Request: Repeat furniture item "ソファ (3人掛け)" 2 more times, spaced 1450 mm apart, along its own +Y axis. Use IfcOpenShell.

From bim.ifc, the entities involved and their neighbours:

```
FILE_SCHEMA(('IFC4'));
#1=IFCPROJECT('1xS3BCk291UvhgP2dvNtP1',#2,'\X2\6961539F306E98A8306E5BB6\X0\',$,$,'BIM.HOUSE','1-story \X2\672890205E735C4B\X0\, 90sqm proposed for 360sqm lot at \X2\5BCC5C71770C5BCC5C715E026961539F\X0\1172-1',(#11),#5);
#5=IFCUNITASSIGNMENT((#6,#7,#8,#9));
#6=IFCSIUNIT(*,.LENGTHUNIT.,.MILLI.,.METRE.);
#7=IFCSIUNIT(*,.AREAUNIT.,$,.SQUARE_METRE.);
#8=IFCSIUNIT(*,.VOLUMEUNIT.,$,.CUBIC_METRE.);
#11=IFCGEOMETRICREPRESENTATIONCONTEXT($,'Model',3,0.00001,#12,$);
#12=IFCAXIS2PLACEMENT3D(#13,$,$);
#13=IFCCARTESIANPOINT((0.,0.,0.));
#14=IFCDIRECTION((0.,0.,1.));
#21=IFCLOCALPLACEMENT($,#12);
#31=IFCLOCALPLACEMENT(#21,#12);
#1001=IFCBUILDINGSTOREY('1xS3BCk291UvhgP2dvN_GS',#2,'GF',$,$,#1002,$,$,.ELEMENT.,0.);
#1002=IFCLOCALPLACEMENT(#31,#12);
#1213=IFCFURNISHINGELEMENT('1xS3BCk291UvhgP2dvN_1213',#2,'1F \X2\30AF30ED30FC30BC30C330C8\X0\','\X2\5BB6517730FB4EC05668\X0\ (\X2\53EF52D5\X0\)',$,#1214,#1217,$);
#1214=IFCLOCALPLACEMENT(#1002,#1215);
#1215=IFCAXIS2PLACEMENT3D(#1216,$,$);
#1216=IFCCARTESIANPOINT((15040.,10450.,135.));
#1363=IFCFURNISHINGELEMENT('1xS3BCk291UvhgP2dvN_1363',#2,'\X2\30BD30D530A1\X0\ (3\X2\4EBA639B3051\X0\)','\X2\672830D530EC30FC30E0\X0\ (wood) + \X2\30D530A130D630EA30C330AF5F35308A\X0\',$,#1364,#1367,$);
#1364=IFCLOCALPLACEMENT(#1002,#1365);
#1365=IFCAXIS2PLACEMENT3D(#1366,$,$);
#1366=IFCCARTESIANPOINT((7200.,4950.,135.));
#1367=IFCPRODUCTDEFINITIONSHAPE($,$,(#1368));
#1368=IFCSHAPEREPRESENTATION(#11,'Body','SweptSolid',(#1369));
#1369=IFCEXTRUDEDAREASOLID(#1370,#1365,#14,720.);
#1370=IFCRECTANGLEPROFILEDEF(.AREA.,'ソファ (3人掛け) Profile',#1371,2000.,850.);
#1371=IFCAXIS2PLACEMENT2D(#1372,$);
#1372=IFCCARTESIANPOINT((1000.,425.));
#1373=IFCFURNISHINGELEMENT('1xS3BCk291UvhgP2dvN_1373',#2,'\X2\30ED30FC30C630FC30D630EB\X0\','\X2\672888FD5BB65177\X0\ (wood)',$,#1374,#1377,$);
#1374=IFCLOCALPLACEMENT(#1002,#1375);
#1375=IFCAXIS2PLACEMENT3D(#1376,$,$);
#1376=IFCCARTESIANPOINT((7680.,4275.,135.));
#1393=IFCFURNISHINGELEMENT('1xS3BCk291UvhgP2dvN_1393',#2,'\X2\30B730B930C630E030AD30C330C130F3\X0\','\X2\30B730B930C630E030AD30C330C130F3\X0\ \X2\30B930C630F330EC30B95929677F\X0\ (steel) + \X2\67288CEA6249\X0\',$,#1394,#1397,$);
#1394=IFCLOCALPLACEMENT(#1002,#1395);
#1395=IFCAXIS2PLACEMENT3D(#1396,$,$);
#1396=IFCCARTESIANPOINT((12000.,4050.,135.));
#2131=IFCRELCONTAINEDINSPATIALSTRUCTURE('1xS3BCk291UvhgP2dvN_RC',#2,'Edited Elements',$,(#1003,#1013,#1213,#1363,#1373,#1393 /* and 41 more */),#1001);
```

```python
import ifcopenshell
import ifcopenshell.api.geometry
import ifcopenshell.api.root
import ifcopenshell.util.element
import ifcopenshell.util.placement
import ifcopenshell.util.unit

model = ifcopenshell.open("bim.ifc")
unit_scale = ifcopenshell.util.unit.calculate_unit_scale(model)


def reuse_history(source, copy):
    """copy_class also copies each property set's owner history, people and application; keep the originals."""
    for rel in copy.IsDefinedBy:
        if rel.is_a("IfcRelDefinesByProperties") and (history := rel.RelatingPropertyDefinition.OwnerHistory):
            rel.RelatingPropertyDefinition.OwnerHistory = source.OwnerHistory
            ifcopenshell.util.element.remove_deep2(model, history)


source = model.by_guid("1xS3BCk291UvhgP2dvN_1363")
base = ifcopenshell.util.placement.get_local_placement(source.ObjectPlacement)
step = base[:3, 1] * 1.45 / unit_scale

for i in range(1, 3):
    copy = ifcopenshell.api.root.copy_class(model, product=source)
    copy.Representation = ifcopenshell.util.element.copy_deep(
        model, source.Representation, exclude=["IfcGeometricRepresentationContext", "IfcRepresentationMap"]
    )
    reuse_history(source, copy)
    matrix = base.copy()
    matrix[:3, 3] += i * step
    print("added at", matrix[:3, 3].round(3) + 0.0)
    ifcopenshell.api.geometry.edit_object_placement(model, product=copy, matrix=matrix, is_si=False)

model.write("bim_updated.ifc")
```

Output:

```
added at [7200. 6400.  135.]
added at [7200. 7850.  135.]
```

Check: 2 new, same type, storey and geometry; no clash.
